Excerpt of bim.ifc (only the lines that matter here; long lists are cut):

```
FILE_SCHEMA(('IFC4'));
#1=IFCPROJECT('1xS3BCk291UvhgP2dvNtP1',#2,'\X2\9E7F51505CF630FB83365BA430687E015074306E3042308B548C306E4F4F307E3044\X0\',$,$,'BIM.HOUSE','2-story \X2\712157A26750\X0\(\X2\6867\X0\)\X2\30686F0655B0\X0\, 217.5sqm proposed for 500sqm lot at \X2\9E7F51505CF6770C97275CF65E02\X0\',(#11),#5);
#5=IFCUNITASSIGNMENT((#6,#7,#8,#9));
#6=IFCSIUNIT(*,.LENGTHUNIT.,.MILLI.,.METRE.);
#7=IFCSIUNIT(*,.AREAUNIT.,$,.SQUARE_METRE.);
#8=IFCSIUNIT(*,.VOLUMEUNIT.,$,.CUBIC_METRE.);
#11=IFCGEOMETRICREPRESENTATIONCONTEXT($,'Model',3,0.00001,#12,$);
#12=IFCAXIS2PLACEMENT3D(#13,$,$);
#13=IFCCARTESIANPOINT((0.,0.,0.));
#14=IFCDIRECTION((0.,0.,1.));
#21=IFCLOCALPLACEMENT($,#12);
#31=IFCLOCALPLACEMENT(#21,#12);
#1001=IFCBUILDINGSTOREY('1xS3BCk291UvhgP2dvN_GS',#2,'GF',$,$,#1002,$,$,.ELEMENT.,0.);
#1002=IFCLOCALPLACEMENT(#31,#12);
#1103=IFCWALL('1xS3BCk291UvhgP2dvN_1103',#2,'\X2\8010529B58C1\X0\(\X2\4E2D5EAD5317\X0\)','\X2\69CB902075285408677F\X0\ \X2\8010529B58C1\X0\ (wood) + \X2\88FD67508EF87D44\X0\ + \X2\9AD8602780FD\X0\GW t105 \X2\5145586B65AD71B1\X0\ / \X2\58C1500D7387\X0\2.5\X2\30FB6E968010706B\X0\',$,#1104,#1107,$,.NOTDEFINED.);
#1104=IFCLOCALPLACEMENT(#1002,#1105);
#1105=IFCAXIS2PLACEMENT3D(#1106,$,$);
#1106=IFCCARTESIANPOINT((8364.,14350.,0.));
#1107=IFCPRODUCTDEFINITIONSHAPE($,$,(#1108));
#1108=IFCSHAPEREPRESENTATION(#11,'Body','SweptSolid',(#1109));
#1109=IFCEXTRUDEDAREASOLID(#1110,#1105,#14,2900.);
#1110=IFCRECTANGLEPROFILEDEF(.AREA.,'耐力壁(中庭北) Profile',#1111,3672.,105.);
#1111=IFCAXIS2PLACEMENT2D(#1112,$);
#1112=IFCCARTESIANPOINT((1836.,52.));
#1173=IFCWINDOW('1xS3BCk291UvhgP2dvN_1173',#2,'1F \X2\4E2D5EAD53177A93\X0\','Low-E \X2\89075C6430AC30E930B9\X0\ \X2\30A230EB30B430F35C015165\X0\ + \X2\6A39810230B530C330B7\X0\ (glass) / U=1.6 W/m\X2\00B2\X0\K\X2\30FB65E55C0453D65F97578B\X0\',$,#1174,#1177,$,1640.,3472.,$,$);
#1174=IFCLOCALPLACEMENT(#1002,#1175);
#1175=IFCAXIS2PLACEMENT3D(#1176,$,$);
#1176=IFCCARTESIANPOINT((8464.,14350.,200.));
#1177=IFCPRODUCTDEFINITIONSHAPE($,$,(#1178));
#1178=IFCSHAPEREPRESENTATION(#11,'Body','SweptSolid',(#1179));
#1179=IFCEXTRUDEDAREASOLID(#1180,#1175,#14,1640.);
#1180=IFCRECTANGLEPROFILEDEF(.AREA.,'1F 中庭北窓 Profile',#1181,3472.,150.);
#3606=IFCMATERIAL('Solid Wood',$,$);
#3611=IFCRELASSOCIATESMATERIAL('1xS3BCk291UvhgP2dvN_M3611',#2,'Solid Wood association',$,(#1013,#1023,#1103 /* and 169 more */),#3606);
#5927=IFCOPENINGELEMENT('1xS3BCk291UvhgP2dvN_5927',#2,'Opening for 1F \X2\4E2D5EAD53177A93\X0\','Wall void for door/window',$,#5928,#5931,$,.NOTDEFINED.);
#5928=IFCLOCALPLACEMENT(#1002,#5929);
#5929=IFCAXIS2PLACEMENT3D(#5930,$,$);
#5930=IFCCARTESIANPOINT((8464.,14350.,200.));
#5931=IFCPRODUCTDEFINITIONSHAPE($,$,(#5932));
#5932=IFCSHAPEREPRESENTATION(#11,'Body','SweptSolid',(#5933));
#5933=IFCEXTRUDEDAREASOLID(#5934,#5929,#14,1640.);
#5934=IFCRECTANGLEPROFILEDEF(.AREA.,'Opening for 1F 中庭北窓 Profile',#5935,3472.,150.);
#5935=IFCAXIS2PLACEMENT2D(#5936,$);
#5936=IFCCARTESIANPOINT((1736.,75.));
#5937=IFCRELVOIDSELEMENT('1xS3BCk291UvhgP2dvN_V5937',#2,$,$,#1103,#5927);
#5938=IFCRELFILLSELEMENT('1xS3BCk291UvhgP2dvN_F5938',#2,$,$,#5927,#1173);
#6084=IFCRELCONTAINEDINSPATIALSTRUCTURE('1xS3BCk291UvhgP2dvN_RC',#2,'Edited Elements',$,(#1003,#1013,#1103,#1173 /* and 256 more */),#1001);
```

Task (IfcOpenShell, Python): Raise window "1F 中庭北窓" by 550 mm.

```python
import numpy as np
import ifcopenshell
import ifcopenshell.api.geometry
import ifcopenshell.util.placement
import ifcopenshell.util.unit

model = ifcopenshell.open("bim.ifc")
unit_scale = ifcopenshell.util.unit.calculate_unit_scale(model)

window = model.by_guid("1xS3BCk291UvhgP2dvN_1173")
opening = window.FillsVoids[0].RelatingOpeningElement
dz = 0.55 / unit_scale

shift = np.array([0.0, 0.0, dz])
# The window is not placed relative to its opening, so move both.
for product in (opening, window):
    matrix = ifcopenshell.util.placement.get_local_placement(product.ObjectPlacement)
    matrix[:3, 3] += shift
    ifcopenshell.api.geometry.edit_object_placement(model, product=product, matrix=matrix, is_si=False)

print(f"moved by {dz * unit_scale:+.3f} m")

model.write("bim_rev.ifc")
```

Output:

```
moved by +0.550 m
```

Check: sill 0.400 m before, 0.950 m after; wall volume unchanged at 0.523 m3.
